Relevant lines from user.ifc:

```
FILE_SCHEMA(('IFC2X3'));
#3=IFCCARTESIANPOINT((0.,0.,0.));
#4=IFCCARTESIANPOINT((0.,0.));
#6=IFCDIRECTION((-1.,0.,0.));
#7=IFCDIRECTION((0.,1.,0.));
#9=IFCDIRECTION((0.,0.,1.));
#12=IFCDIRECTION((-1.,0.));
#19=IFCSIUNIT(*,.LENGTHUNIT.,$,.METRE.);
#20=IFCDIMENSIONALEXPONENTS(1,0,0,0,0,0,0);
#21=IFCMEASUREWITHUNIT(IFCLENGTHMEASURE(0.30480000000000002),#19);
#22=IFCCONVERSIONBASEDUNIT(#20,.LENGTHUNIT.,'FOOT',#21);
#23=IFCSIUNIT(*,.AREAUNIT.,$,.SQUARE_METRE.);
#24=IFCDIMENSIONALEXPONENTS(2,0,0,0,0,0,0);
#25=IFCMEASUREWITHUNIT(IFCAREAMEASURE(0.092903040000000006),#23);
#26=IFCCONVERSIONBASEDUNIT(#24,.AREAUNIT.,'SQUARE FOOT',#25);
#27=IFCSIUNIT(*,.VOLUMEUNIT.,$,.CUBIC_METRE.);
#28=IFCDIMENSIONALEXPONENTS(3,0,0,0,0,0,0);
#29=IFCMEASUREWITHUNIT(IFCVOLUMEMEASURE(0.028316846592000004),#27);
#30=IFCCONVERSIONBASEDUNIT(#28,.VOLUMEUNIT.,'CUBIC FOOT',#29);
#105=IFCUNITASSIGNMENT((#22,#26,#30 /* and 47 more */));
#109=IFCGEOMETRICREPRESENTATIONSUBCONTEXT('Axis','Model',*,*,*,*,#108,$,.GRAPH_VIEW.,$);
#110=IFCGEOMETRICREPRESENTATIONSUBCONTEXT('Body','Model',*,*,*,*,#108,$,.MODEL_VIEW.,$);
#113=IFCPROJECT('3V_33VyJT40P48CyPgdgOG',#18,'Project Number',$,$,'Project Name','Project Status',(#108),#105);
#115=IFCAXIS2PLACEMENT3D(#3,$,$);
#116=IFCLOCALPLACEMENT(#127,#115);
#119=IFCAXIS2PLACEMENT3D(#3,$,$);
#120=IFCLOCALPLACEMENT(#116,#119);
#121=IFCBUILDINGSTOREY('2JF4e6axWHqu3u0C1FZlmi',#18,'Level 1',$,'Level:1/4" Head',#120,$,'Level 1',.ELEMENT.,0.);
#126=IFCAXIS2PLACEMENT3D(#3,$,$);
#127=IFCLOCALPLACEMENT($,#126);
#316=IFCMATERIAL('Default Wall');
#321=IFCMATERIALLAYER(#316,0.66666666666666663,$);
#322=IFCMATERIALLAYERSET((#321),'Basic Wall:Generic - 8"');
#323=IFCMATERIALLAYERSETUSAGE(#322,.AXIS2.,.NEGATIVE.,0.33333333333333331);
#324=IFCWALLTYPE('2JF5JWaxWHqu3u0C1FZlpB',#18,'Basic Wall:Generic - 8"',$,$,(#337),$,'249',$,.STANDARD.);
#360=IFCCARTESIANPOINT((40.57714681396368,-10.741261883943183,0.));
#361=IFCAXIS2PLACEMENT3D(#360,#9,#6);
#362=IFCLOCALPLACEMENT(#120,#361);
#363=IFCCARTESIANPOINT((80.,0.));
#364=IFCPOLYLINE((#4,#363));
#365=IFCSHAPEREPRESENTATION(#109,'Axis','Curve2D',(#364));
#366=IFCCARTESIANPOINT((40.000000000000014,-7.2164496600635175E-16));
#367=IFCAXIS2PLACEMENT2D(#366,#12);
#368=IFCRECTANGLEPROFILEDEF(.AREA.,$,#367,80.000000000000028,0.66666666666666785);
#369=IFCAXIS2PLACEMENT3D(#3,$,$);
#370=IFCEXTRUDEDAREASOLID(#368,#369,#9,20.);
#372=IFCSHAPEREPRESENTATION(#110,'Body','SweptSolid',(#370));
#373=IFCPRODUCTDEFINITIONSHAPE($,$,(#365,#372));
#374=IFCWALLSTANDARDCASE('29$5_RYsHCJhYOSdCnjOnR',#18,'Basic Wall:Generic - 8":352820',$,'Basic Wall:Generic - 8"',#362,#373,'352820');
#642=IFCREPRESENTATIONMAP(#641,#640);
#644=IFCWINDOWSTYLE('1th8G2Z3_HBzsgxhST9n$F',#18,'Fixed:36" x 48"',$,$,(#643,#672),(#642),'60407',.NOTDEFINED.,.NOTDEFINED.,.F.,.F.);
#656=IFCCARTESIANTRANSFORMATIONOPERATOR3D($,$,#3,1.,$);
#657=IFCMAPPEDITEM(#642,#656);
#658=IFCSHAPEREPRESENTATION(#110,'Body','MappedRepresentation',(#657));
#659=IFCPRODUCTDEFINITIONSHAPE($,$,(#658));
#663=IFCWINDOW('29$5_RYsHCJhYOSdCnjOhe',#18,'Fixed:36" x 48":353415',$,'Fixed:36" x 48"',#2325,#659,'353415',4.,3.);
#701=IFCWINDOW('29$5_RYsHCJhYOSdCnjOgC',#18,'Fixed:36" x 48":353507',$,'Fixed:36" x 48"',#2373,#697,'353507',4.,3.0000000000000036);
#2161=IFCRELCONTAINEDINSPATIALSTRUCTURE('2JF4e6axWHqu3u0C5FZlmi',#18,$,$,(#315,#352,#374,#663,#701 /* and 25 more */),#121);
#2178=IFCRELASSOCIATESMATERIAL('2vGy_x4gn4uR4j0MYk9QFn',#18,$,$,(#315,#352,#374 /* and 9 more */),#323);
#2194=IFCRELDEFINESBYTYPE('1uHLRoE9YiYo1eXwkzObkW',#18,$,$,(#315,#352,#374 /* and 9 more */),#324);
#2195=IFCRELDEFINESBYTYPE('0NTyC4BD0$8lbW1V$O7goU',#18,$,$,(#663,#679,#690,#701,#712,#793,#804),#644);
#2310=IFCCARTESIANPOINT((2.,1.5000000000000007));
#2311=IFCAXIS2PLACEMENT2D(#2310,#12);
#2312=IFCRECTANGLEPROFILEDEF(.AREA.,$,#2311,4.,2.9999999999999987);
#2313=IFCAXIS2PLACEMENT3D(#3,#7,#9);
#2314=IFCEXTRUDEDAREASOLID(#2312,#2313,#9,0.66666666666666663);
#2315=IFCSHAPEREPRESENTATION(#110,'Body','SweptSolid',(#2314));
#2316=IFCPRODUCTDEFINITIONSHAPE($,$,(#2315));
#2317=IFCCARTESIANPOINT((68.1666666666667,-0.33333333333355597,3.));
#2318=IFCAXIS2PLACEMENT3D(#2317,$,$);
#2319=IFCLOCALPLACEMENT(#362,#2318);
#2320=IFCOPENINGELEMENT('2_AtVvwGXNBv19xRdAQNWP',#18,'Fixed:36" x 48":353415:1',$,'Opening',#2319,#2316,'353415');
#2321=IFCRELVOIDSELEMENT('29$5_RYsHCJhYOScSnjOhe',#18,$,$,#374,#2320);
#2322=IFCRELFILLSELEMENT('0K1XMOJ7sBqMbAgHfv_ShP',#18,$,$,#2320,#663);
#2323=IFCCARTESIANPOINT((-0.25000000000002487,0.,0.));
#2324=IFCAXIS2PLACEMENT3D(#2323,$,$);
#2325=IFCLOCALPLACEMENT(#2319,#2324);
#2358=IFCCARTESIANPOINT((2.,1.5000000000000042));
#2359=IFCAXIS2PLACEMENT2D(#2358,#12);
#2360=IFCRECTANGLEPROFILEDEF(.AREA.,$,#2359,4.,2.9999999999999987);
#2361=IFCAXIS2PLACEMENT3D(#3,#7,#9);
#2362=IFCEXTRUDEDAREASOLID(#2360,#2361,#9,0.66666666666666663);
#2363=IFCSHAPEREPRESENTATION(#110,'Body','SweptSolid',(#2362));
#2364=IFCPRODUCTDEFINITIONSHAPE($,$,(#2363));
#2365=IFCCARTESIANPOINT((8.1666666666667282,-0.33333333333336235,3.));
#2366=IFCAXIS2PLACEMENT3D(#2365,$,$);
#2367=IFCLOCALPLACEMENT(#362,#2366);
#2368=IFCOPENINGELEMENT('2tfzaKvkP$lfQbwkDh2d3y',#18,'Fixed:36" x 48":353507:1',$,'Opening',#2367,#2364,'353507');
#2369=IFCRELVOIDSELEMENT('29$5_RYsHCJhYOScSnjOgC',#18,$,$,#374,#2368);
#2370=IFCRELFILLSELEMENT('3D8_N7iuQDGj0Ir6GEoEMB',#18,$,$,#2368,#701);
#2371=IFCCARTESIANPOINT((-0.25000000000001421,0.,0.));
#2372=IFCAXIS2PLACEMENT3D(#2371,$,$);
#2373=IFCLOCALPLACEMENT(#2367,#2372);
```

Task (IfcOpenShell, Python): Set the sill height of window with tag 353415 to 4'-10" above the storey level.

```python
import numpy as np
import ifcopenshell
import ifcopenshell.api.geometry
import ifcopenshell.geom
import ifcopenshell.util.element
import ifcopenshell.util.placement
import ifcopenshell.util.shape
import ifcopenshell.util.unit

model = ifcopenshell.open("user.ifc")
unit_scale = ifcopenshell.util.unit.calculate_unit_scale(model)

window = model.by_id(663)
opening = window.FillsVoids[0].RelatingOpeningElement
storey = ifcopenshell.util.element.get_container(window, ifc_class="IfcBuildingStorey")
level = ifcopenshell.util.placement.get_local_placement(storey.ObjectPlacement)[2, 3]

# The opening's origin need not be at the sill, so measure its lowest point.
shape = ifcopenshell.geom.create_shape(ifcopenshell.geom.settings(), opening)
bottom = ifcopenshell.util.shape.get_shape_bottom_elevation(shape, shape.geometry) / unit_scale
dz = level + 58 * 0.0254 / unit_scale - bottom

shift = np.array([0.0, 0.0, dz])
# The window is placed relative to its opening, so it follows when the opening moves.
matrix = ifcopenshell.util.placement.get_local_placement(opening.ObjectPlacement)
matrix[:3, 3] += shift
ifcopenshell.api.geometry.edit_object_placement(
    model, product=opening, matrix=matrix, is_si=False, should_transform_children=True
)

print(f"moved by {dz * unit_scale:+.3f} m")

model.write("user_rev.ifc")
```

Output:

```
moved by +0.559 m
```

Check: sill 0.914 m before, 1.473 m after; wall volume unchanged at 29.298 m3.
